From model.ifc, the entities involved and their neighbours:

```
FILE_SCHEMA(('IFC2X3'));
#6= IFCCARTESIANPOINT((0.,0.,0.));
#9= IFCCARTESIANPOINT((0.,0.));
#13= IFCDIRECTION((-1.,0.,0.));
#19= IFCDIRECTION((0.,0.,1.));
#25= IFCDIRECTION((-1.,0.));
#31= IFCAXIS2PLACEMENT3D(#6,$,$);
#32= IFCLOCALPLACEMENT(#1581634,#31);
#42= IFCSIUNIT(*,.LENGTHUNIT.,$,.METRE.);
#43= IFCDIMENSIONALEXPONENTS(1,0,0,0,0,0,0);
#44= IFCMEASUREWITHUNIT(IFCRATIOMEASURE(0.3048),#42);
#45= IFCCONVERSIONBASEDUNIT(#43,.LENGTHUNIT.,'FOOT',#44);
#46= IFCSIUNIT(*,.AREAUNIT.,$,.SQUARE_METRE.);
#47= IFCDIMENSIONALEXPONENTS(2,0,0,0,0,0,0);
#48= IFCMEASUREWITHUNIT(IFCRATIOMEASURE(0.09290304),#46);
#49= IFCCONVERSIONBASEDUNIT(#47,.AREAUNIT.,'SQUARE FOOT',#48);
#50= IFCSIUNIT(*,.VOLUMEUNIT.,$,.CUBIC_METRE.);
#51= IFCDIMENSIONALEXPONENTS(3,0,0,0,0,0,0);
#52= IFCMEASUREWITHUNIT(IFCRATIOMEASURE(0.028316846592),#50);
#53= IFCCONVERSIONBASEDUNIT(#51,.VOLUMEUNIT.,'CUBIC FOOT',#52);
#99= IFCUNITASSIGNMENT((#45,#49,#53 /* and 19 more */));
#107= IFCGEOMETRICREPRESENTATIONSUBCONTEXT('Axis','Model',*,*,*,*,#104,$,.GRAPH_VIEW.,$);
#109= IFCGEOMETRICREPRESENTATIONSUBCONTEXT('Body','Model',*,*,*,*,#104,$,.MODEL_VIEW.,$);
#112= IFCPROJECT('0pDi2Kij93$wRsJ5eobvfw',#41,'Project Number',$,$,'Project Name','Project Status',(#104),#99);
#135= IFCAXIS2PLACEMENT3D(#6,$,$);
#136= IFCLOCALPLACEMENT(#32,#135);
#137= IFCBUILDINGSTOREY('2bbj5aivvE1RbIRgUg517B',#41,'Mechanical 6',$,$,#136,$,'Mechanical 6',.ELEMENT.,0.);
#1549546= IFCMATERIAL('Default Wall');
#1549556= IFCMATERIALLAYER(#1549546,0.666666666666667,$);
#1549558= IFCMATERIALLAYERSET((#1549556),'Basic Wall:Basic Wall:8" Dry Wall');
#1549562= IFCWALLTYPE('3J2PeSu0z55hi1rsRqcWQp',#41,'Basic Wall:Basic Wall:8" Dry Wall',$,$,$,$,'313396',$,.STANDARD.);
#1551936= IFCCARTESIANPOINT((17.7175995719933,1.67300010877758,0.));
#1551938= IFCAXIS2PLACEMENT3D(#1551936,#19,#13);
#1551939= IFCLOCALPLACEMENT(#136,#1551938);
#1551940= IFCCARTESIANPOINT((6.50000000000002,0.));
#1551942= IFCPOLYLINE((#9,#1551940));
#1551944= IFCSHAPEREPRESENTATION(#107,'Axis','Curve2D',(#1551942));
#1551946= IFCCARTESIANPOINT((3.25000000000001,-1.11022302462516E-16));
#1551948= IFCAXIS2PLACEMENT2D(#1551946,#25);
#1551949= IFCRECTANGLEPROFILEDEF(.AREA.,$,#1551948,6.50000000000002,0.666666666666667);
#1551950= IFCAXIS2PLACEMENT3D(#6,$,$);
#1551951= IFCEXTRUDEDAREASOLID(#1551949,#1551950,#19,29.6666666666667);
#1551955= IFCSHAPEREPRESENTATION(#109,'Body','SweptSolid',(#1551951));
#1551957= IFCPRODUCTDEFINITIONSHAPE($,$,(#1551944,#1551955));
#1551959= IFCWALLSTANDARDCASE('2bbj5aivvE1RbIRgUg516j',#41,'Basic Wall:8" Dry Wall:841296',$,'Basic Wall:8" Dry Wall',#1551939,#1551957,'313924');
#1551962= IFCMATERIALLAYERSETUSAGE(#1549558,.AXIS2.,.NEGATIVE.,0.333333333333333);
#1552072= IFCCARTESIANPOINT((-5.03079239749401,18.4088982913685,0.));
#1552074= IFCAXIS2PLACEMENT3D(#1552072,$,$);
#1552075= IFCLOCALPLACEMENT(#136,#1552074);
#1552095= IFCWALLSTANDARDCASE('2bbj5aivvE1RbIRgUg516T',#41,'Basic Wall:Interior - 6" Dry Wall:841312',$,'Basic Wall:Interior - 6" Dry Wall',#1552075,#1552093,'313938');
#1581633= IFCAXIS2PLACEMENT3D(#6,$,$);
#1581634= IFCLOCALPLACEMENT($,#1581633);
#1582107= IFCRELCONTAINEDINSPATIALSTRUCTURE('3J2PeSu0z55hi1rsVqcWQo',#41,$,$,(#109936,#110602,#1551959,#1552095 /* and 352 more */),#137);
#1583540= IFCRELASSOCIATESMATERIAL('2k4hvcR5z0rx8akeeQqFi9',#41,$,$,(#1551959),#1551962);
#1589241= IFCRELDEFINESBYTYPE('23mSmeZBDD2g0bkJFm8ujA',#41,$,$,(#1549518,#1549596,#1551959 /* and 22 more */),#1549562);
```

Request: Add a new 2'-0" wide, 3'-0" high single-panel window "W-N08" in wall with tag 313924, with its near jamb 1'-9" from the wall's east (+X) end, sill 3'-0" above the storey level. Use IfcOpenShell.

```python
import numpy as np
import ifcopenshell
import ifcopenshell.api.feature
import ifcopenshell.api.geometry
import ifcopenshell.api.root
import ifcopenshell.api.spatial
import ifcopenshell.api.type
import ifcopenshell.geom
import ifcopenshell.util.element
import ifcopenshell.util.placement
import ifcopenshell.util.representation
import ifcopenshell.util.shape
import ifcopenshell.util.unit

model = ifcopenshell.open("model.ifc")
unit_scale = ifcopenshell.util.unit.calculate_unit_scale(model)
settings = ifcopenshell.geom.settings()


def volume(element):
    """Net volume in cubic metres, openings subtracted."""
    shape = ifcopenshell.geom.create_shape(settings, element)
    return ifcopenshell.util.shape.get_volume(shape.geometry)


wall = model.by_id(1551959)
storey = ifcopenshell.util.element.get_container(wall, ifc_class="IfcBuildingStorey")
context = ifcopenshell.util.representation.get_context(model, "Model", "Body", "MODEL_VIEW")
before = volume(wall)

width, height, from_end, sill = 0.6096, 0.9144, 0.5334, 0.9144  # metres

# The wall runs along its own X axis, and the end named is its -X end.
wall_shape = ifcopenshell.geom.create_shape(settings, wall)
x, y, z = ifcopenshell.util.shape.get_vertices(wall_shape.geometry).T
start = x.min() + from_end
face, thickness = float(y.min()), float(y.max() - y.min())
wall_matrix = ifcopenshell.util.placement.get_local_placement(wall.ObjectPlacement)
level = ifcopenshell.util.placement.get_local_placement(storey.ObjectPlacement)[2, 3]


def in_wall(x, y):
    """Placement at x, y metres in the wall's axes, at sill height."""
    matrix = wall_matrix.copy()
    matrix[:, 3] = wall_matrix @ np.array([x / unit_scale, y / unit_scale, 0.0, 1.0])
    matrix[2, 3] = level + sill / unit_scale
    return matrix


# Opening: a box that overshoots both wall faces by 50 mm.
opening = ifcopenshell.api.root.create_entity(model, ifc_class="IfcOpeningElement")
box = ifcopenshell.api.geometry.add_wall_representation(
    model, context=context, length=width, height=height, thickness=thickness + 0.1
)
ifcopenshell.api.geometry.assign_representation(model, product=opening, representation=box)
ifcopenshell.api.geometry.edit_object_placement(model, product=opening, matrix=in_wall(start, face - 0.05), is_si=False)
ifcopenshell.api.feature.add_feature(model, feature=opening, element=wall)

window = ifcopenshell.api.root.create_entity(model, ifc_class="IfcWindow", name="W-N08")
window.OverallWidth, window.OverallHeight = width / unit_scale, height / unit_scale
body = ifcopenshell.api.geometry.add_window_representation(
    model,
    context=context,
    overall_width=window.OverallWidth,
    overall_height=window.OverallHeight,
    partition_type="SINGLE_PANEL",
)
ifcopenshell.api.geometry.assign_representation(model, product=window, representation=body)
ifcopenshell.api.spatial.assign_container(model, products=[window], relating_structure=storey)
fills = ifcopenshell.api.feature.add_filling(model, opening=opening, element=window)
fills.OwnerHistory = window.OwnerHistory  # required in IFC2X3

# IFC2X3 keeps the operation on the window style.
style = ifcopenshell.api.root.create_entity(model, ifc_class="IfcWindowStyle", name="W-N08")
style.OperationType, style.ConstructionType = "SINGLE_PANEL", "NOTDEFINED"
style.ParameterTakesPrecedence = style.Sizeable = False
ifcopenshell.api.type.assign_type(model, related_objects=[window], relating_type=style)

# Centre the window in the wall's thickness.
ifcopenshell.api.geometry.edit_object_placement(model, product=window, matrix=in_wall(start, face), is_si=False)
window_shape = ifcopenshell.geom.create_shape(settings, window)
depth = ifcopenshell.util.shape.get_vertices(window_shape.geometry)[:, 1]
offset = face + thickness / 2 - (depth.min() + depth.max()) / 2
ifcopenshell.api.geometry.edit_object_placement(model, product=window, matrix=in_wall(start, offset), is_si=False)

after = volume(wall)

print(f"wall volume {before:.3f} -> {after:.3f} m3")

model.write("model_edited.ifc")
```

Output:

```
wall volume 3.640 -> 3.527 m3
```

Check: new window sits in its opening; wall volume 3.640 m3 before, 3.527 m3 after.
